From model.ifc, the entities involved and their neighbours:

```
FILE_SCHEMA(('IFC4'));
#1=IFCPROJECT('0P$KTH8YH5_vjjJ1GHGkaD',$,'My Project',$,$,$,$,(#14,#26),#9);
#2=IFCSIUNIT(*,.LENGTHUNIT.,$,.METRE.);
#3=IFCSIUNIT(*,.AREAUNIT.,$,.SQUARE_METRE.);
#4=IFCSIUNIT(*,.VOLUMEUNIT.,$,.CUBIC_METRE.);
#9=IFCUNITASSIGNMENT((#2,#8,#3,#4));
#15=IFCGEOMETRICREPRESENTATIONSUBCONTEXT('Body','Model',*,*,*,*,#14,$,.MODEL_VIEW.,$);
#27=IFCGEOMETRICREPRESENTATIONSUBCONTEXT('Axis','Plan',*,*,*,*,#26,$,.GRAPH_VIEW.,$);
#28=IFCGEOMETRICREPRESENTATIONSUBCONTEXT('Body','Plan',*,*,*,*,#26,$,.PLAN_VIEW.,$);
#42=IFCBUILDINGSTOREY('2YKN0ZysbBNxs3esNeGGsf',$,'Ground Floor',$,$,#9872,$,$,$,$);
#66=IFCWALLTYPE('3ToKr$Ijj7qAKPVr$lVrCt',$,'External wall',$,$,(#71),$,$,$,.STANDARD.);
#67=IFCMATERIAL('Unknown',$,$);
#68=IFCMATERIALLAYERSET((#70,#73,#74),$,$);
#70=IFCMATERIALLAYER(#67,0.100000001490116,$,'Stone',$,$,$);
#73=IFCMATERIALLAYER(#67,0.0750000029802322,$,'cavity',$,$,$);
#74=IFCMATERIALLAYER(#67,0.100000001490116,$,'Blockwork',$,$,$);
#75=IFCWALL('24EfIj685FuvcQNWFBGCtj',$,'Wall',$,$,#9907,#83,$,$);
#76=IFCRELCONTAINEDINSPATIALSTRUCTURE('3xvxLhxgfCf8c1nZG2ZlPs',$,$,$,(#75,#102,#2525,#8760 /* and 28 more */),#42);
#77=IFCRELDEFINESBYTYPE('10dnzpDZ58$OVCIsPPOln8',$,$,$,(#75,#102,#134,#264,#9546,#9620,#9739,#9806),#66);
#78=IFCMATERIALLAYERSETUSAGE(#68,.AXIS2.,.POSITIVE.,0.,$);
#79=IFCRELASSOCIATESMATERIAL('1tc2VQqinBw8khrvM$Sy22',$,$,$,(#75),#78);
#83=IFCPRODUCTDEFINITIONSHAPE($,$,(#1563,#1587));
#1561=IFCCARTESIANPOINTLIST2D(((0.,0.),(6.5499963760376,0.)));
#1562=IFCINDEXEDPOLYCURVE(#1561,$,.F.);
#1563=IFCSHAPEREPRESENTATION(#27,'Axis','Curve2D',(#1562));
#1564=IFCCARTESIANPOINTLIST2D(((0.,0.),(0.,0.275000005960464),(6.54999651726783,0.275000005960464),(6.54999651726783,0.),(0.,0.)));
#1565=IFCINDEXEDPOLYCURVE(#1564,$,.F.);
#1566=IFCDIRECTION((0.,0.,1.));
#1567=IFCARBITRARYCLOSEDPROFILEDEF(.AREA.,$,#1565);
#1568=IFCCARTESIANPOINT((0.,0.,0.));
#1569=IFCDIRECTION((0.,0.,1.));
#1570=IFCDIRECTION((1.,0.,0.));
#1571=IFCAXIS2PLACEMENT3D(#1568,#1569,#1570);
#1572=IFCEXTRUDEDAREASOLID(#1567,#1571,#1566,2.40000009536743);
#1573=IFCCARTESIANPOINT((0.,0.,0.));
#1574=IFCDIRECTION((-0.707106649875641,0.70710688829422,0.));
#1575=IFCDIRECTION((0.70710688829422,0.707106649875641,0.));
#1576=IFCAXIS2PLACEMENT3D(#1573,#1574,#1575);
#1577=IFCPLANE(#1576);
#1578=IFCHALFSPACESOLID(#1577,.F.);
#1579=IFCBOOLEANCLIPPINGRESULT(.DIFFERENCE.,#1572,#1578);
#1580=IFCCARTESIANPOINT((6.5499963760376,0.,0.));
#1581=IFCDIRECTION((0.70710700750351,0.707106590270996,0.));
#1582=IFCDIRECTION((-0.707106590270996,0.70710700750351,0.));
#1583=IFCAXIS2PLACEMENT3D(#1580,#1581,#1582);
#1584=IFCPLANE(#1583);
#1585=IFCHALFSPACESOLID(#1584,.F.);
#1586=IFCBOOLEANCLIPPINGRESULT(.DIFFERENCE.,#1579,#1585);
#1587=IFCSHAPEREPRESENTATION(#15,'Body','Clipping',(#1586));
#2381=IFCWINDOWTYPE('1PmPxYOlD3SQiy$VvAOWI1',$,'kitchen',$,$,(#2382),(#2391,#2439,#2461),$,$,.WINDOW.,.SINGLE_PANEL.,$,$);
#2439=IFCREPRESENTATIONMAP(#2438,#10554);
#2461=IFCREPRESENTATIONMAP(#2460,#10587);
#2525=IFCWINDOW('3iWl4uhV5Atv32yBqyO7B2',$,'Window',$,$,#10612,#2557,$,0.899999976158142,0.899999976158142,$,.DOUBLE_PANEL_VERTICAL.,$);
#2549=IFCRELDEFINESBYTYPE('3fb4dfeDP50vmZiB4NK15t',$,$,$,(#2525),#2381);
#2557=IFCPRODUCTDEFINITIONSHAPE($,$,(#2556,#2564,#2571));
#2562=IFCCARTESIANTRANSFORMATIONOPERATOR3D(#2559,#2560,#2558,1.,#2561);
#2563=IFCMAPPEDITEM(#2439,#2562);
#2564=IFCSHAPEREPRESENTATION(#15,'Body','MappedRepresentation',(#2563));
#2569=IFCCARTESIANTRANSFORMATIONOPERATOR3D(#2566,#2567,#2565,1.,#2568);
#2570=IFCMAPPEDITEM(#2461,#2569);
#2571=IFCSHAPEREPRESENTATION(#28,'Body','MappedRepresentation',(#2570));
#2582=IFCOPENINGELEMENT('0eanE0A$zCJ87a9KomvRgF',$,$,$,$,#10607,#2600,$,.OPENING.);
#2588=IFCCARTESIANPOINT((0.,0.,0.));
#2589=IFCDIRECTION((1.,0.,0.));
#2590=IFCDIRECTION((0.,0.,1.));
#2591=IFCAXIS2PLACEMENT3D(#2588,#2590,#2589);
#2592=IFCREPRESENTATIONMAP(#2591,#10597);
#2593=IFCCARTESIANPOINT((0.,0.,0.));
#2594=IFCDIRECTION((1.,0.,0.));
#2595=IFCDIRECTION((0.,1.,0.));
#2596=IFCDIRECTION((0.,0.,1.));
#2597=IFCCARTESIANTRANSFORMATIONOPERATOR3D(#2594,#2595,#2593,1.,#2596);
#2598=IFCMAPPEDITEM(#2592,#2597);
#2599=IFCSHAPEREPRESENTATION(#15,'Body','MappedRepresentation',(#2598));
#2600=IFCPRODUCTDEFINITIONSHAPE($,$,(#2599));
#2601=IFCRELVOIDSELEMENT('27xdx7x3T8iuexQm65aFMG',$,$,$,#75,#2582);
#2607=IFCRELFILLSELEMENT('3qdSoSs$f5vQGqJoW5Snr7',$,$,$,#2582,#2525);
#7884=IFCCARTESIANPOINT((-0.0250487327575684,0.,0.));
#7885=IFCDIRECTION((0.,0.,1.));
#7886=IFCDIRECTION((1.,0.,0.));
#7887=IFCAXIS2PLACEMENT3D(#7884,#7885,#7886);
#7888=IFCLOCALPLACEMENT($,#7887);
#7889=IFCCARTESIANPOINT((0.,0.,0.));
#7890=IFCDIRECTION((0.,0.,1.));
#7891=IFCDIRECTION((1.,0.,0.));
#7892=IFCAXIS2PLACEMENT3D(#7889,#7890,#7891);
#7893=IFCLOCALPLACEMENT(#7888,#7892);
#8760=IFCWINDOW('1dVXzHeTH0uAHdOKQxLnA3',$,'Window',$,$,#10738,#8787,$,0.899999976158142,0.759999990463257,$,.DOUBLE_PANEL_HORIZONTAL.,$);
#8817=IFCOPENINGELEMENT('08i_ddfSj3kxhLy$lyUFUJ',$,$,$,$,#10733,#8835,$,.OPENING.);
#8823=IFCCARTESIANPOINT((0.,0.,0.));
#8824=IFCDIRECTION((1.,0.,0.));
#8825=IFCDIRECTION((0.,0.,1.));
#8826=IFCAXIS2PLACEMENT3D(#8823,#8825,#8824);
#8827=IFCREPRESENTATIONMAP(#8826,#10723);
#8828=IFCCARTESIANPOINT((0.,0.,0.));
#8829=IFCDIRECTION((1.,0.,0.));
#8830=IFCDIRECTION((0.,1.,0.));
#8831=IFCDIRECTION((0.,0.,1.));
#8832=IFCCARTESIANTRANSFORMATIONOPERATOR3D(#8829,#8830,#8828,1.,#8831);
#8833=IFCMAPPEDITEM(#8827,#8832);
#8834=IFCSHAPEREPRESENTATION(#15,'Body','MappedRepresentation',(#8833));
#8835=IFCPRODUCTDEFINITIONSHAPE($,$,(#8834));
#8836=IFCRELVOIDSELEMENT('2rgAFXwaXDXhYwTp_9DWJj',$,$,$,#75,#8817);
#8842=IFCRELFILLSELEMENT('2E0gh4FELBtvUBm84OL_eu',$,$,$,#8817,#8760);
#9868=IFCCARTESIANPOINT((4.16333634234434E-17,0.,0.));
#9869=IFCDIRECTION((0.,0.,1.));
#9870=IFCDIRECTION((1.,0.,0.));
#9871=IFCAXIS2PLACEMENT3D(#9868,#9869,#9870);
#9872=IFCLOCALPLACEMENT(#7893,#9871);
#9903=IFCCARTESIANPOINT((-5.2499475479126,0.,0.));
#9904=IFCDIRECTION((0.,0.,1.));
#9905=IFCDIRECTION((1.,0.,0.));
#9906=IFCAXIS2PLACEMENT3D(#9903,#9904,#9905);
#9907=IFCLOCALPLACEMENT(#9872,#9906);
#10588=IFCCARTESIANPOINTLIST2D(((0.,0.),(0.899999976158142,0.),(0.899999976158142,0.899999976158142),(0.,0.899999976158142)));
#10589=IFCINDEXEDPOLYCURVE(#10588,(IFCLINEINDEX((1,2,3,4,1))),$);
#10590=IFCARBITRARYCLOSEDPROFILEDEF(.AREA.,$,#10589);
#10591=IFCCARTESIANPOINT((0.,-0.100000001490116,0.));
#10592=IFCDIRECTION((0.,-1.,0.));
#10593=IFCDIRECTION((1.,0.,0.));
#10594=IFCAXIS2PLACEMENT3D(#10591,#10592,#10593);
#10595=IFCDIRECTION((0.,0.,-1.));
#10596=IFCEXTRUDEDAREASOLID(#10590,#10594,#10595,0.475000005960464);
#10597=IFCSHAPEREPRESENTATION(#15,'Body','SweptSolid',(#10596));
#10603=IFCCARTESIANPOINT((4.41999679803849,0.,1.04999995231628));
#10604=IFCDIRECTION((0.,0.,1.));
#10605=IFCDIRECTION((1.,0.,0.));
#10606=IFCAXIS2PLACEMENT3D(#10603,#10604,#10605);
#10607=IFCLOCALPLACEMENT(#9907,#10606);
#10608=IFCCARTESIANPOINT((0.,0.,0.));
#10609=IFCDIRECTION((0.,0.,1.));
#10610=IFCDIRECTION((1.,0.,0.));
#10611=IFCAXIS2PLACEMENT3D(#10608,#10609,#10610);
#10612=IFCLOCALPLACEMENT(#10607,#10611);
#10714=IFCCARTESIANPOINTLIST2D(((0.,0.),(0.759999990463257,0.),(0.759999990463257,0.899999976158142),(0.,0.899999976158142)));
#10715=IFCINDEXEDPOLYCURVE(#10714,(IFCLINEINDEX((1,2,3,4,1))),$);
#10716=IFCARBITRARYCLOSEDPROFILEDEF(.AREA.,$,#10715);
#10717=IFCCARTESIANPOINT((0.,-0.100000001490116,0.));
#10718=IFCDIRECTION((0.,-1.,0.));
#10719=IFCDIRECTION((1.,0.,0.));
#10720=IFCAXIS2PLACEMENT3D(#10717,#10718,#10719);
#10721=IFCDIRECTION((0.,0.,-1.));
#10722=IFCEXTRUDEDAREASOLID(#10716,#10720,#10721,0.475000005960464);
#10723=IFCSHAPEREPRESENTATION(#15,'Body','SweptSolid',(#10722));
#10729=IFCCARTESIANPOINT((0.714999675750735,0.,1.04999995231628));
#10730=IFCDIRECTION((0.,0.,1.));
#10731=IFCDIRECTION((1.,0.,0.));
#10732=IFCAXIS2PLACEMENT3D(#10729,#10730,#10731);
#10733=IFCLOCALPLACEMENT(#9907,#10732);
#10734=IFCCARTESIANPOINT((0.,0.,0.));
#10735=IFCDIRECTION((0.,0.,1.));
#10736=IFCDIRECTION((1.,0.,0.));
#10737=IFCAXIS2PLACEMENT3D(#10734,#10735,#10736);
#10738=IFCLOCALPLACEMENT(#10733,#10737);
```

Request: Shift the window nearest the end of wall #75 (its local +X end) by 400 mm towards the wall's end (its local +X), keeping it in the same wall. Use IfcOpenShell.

```python
import ifcopenshell
import ifcopenshell.api.geometry
import ifcopenshell.util.placement

model = ifcopenshell.open("model.ifc")

window = model.by_guid("3iWl4uhV5Atv32yBqyO7B2")
opening = window.FillsVoids[0].RelatingOpeningElement
wall = opening.VoidsElements[0].RelatingBuildingElement

wall_matrix = ifcopenshell.util.placement.get_local_placement(wall.ObjectPlacement)
shift = wall_matrix[:3, 0] * 0.4
before = ifcopenshell.util.placement.get_local_placement(window.ObjectPlacement)[:3, 3].copy()

# The window is placed relative to its opening, so it follows when the opening moves.
matrix = ifcopenshell.util.placement.get_local_placement(opening.ObjectPlacement)
matrix[:3, 3] += shift
ifcopenshell.api.geometry.edit_object_placement(
    model, product=opening, matrix=matrix, is_si=False, should_transform_children=True
)

after = ifcopenshell.util.placement.get_local_placement(window.ObjectPlacement)[:3, 3]
print("window moved by", (after - before).round(3) + 0.0)

model.write("model_rev.ifc")
```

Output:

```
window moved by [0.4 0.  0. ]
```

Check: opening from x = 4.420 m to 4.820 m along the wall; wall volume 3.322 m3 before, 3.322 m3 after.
